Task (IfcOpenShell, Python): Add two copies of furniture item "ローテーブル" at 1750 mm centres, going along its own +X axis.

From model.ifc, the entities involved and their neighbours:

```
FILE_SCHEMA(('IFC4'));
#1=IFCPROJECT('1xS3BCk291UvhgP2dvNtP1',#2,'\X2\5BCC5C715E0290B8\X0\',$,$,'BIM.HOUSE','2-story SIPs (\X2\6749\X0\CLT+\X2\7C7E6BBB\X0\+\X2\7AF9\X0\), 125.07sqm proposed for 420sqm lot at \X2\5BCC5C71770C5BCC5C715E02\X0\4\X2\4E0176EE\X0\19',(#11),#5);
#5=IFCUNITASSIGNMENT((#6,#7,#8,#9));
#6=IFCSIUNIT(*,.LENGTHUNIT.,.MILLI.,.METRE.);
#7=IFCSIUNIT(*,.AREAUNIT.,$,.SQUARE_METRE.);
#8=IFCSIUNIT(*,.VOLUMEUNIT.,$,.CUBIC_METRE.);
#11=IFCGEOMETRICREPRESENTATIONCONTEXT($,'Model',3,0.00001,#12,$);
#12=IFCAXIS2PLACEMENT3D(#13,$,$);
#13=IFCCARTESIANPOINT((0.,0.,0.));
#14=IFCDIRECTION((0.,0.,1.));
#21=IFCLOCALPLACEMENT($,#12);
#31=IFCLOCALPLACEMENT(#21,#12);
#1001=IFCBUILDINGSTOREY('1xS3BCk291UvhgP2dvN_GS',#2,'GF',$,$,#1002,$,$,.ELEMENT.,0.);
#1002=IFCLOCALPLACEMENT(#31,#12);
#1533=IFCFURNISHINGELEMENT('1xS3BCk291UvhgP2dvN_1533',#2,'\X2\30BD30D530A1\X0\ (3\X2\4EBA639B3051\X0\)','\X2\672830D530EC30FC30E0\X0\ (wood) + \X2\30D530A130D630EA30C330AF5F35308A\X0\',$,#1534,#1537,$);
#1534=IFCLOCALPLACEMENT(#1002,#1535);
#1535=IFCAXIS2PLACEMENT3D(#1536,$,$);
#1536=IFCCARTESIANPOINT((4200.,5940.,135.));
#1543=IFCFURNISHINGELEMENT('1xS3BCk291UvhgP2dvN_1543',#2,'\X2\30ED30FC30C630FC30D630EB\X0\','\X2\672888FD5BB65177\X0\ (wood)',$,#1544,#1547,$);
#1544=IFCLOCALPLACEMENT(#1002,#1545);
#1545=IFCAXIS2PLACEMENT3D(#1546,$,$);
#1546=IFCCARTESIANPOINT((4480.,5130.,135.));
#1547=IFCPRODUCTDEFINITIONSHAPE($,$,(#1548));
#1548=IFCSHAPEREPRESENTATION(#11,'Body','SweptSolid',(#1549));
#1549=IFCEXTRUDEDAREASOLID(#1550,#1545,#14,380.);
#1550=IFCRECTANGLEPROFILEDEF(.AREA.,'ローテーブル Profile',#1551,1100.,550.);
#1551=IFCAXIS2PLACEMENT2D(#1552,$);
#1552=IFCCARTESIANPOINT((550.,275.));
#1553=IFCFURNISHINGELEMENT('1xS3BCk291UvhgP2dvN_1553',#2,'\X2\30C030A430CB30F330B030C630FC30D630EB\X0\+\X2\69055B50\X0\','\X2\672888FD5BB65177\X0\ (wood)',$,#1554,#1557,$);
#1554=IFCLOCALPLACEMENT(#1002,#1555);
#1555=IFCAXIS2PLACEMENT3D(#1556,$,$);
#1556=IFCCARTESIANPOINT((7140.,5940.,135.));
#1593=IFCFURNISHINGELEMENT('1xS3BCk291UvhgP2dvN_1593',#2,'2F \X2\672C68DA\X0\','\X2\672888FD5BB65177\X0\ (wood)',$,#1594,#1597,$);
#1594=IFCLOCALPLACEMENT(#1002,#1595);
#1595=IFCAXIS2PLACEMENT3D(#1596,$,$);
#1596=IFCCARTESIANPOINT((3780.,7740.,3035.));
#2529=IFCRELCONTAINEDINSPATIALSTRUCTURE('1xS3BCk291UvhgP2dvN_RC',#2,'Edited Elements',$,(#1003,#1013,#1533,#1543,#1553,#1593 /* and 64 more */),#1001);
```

```python
import ifcopenshell
import ifcopenshell.api.geometry
import ifcopenshell.api.root
import ifcopenshell.util.element
import ifcopenshell.util.placement
import ifcopenshell.util.unit

model = ifcopenshell.open("model.ifc")
unit_scale = ifcopenshell.util.unit.calculate_unit_scale(model)


def reuse_history(source, copy):
    """copy_class also copies each property set's owner history, people and application; keep the originals."""
    for rel in copy.IsDefinedBy:
        if rel.is_a("IfcRelDefinesByProperties") and (history := rel.RelatingPropertyDefinition.OwnerHistory):
            rel.RelatingPropertyDefinition.OwnerHistory = source.OwnerHistory
            ifcopenshell.util.element.remove_deep2(model, history)


source = model.by_guid("1xS3BCk291UvhgP2dvN_1543")
base = ifcopenshell.util.placement.get_local_placement(source.ObjectPlacement)
step = base[:3, 0] * 1.75 / unit_scale

for i in range(1, 3):
    copy = ifcopenshell.api.root.copy_class(model, product=source)
    copy.Representation = ifcopenshell.util.element.copy_deep(
        model, source.Representation, exclude=["IfcGeometricRepresentationContext", "IfcRepresentationMap"]
    )
    reuse_history(source, copy)
    matrix = base.copy()
    matrix[:3, 3] += i * step
    print("added at", matrix[:3, 3].round(3) + 0.0)
    ifcopenshell.api.geometry.edit_object_placement(model, product=copy, matrix=matrix, is_si=False)

model.write("model-out.ifc")
```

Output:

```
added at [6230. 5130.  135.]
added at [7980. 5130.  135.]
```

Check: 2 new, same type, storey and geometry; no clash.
